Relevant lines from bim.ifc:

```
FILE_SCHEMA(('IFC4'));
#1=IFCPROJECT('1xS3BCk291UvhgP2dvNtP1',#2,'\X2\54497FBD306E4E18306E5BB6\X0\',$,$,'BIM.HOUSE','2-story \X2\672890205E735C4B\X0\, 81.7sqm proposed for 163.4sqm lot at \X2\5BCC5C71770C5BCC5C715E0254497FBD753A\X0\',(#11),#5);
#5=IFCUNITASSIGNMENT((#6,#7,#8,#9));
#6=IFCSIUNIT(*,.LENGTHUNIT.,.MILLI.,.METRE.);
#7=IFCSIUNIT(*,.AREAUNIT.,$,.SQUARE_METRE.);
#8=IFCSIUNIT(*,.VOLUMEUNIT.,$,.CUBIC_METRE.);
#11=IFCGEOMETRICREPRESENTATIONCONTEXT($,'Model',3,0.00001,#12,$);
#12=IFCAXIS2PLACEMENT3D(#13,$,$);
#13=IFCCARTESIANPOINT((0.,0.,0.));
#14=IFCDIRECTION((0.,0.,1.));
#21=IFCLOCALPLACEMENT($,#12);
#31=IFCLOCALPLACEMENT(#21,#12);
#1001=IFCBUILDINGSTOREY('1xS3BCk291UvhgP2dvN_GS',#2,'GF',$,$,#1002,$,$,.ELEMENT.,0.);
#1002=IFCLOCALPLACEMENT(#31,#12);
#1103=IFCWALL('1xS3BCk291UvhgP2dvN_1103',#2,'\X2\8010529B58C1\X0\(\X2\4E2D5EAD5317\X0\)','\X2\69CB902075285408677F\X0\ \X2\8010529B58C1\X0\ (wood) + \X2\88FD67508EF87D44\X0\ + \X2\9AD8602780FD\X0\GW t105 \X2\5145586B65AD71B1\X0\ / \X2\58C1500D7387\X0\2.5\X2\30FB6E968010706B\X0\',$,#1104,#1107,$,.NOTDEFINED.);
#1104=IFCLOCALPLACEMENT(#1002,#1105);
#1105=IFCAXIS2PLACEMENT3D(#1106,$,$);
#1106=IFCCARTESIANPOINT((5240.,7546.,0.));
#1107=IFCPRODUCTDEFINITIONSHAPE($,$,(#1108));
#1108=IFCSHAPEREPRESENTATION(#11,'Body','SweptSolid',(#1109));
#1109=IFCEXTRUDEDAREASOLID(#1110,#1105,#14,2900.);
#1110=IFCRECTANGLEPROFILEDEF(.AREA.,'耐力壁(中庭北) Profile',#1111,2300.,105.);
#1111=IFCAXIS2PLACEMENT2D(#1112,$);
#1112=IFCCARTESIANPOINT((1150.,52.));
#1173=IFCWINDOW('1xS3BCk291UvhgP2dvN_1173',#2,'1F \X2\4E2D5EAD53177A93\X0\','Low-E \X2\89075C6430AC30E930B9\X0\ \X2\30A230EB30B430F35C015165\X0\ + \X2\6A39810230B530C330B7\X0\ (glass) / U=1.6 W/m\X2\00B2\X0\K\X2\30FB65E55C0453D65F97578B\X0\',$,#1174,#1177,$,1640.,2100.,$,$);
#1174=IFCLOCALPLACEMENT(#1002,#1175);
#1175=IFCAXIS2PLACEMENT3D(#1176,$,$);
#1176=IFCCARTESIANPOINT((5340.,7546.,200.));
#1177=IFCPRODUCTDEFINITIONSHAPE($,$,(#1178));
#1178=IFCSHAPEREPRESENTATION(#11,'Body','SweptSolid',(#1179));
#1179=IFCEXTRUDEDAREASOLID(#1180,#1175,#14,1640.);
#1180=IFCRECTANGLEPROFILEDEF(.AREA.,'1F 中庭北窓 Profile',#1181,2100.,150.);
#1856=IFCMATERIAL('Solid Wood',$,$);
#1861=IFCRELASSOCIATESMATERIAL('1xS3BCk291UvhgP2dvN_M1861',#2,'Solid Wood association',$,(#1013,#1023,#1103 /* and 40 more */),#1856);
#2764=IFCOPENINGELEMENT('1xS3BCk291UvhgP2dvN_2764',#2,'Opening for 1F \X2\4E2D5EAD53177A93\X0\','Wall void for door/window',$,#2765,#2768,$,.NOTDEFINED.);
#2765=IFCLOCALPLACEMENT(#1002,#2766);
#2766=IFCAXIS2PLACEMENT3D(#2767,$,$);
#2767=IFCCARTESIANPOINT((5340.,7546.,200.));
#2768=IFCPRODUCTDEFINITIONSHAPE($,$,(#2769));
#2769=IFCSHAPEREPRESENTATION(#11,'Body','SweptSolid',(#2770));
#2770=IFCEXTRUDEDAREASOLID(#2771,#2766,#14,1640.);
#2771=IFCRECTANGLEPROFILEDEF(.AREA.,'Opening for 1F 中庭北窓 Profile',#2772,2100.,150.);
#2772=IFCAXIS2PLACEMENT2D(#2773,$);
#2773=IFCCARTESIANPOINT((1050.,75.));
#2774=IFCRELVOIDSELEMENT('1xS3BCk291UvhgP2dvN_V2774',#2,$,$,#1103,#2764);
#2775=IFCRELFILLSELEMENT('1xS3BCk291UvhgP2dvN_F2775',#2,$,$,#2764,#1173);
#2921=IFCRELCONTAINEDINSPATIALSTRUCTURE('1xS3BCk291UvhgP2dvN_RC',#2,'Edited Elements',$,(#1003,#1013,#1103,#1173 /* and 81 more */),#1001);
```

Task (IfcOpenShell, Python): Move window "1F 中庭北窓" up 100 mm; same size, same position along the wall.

```python
import numpy as np
import ifcopenshell
import ifcopenshell.api.geometry
import ifcopenshell.util.placement
import ifcopenshell.util.unit

model = ifcopenshell.open("bim.ifc")
unit_scale = ifcopenshell.util.unit.calculate_unit_scale(model)

window = model.by_id(1173)
opening = window.FillsVoids[0].RelatingOpeningElement
dz = 100.0

shift = np.array([0.0, 0.0, dz])
# The window is not placed relative to its opening, so move both.
for product in (opening, window):
    matrix = ifcopenshell.util.placement.get_local_placement(product.ObjectPlacement)
    matrix[:3, 3] += shift
    ifcopenshell.api.geometry.edit_object_placement(model, product=product, matrix=matrix, is_si=False)

print(f"moved by {dz * unit_scale:+.3f} m")

model.write("bim_updated.ifc")
```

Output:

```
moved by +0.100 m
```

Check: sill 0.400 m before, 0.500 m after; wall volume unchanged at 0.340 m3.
